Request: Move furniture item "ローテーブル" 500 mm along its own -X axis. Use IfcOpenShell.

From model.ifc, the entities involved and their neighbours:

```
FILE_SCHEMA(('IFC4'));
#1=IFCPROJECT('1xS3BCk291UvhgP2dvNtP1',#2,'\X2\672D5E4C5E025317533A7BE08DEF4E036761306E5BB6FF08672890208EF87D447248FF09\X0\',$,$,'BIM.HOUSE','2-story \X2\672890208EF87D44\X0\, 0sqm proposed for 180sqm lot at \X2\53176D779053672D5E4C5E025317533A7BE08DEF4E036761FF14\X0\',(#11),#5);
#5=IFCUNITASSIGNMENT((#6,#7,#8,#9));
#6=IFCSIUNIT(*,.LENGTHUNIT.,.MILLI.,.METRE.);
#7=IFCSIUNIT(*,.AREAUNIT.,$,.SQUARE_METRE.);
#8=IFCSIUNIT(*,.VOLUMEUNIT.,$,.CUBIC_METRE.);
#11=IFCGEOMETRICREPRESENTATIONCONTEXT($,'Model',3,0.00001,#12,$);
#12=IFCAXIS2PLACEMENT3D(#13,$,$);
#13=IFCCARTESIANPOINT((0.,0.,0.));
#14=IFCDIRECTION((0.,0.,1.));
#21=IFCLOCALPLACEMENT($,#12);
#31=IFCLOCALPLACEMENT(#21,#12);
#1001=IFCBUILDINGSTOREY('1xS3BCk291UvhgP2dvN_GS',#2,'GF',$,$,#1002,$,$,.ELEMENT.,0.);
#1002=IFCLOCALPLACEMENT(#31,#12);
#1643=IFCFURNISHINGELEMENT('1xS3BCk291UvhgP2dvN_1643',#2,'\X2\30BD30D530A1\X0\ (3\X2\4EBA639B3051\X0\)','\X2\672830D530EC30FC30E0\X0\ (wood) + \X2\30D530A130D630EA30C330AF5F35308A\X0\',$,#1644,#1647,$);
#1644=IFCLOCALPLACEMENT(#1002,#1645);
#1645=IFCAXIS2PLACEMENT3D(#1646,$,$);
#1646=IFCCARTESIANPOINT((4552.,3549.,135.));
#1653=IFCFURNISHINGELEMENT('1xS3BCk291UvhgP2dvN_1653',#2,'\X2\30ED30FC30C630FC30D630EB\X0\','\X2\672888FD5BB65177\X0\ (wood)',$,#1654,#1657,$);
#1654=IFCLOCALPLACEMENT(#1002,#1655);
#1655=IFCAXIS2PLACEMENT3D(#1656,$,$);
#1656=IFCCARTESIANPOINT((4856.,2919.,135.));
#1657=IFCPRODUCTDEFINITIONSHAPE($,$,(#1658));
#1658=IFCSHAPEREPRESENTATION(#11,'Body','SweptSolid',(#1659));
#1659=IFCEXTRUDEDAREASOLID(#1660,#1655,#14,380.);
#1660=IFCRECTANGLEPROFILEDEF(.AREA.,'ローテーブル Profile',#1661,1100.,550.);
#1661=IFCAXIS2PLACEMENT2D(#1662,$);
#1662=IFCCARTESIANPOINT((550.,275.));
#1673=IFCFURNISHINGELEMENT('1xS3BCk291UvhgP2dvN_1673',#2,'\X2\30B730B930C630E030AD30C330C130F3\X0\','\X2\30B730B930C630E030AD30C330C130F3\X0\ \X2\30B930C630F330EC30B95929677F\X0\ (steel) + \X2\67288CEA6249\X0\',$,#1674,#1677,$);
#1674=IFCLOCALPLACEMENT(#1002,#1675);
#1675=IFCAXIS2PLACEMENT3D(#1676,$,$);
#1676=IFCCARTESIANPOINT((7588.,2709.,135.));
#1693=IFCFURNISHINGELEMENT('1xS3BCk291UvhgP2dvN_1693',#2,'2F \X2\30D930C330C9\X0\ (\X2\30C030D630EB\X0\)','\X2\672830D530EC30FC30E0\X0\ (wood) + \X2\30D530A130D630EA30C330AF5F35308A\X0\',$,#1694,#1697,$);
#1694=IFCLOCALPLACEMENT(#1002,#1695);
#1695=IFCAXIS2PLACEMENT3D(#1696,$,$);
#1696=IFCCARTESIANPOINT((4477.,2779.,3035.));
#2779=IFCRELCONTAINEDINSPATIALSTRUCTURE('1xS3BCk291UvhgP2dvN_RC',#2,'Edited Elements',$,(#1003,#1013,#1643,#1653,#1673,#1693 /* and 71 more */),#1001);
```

```python
import ifcopenshell
import ifcopenshell.api.geometry
import ifcopenshell.util.placement
import ifcopenshell.util.unit

model = ifcopenshell.open("model.ifc")
unit_scale = ifcopenshell.util.unit.calculate_unit_scale(model)

item = model.by_id(1653)
matrix = ifcopenshell.util.placement.get_local_placement(item.ObjectPlacement)
matrix[:3, 3] -= matrix[:3, 0] * 0.5 / unit_scale
ifcopenshell.api.geometry.edit_object_placement(model, product=item, matrix=matrix, is_si=False)

print(ifcopenshell.util.placement.get_local_placement(item.ObjectPlacement).round(3) + 0.0)

model.write("model_rev.ifc")
```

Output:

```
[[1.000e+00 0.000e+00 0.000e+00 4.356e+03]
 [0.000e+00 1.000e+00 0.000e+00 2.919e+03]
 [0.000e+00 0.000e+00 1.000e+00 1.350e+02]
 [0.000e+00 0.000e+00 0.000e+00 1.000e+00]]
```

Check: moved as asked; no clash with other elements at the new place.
